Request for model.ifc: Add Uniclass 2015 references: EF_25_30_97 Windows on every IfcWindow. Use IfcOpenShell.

First a look at what the model holds.

```python
import ifcopenshell

model = ifcopenshell.open("model.ifc")
print(model.schema)
print("classifications:", [c.Name for c in model.by_type("IfcClassification")])
for ifc_class in ("IfcDoor", "IfcRoof", "IfcStair", "IfcWall", "IfcWindow"):
    print(ifc_class, len(model.by_type(ifc_class)))
```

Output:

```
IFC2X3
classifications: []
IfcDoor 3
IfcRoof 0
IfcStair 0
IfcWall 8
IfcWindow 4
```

```python
import ifcopenshell
import ifcopenshell.api.classification

model = ifcopenshell.open("model.ifc")

# IFC2X3 requires Source and Edition and has no link from the project to the system.
system = model.create_entity("IfcClassification", Source="NBS", Edition="2015", Name="Uniclass 2015")

codes = {
    "IfcWindow": ("EF_25_30_97", "Windows"),
}
for ifc_class, (code, name) in codes.items():
    products = model.by_type(ifc_class)
    ifcopenshell.api.classification.add_reference(
        model, products=products, classification=system, identification=code, name=name
    )
    print(code, len(products))

model.write("model_v2.ifc")
```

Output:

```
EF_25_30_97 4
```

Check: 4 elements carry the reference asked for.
